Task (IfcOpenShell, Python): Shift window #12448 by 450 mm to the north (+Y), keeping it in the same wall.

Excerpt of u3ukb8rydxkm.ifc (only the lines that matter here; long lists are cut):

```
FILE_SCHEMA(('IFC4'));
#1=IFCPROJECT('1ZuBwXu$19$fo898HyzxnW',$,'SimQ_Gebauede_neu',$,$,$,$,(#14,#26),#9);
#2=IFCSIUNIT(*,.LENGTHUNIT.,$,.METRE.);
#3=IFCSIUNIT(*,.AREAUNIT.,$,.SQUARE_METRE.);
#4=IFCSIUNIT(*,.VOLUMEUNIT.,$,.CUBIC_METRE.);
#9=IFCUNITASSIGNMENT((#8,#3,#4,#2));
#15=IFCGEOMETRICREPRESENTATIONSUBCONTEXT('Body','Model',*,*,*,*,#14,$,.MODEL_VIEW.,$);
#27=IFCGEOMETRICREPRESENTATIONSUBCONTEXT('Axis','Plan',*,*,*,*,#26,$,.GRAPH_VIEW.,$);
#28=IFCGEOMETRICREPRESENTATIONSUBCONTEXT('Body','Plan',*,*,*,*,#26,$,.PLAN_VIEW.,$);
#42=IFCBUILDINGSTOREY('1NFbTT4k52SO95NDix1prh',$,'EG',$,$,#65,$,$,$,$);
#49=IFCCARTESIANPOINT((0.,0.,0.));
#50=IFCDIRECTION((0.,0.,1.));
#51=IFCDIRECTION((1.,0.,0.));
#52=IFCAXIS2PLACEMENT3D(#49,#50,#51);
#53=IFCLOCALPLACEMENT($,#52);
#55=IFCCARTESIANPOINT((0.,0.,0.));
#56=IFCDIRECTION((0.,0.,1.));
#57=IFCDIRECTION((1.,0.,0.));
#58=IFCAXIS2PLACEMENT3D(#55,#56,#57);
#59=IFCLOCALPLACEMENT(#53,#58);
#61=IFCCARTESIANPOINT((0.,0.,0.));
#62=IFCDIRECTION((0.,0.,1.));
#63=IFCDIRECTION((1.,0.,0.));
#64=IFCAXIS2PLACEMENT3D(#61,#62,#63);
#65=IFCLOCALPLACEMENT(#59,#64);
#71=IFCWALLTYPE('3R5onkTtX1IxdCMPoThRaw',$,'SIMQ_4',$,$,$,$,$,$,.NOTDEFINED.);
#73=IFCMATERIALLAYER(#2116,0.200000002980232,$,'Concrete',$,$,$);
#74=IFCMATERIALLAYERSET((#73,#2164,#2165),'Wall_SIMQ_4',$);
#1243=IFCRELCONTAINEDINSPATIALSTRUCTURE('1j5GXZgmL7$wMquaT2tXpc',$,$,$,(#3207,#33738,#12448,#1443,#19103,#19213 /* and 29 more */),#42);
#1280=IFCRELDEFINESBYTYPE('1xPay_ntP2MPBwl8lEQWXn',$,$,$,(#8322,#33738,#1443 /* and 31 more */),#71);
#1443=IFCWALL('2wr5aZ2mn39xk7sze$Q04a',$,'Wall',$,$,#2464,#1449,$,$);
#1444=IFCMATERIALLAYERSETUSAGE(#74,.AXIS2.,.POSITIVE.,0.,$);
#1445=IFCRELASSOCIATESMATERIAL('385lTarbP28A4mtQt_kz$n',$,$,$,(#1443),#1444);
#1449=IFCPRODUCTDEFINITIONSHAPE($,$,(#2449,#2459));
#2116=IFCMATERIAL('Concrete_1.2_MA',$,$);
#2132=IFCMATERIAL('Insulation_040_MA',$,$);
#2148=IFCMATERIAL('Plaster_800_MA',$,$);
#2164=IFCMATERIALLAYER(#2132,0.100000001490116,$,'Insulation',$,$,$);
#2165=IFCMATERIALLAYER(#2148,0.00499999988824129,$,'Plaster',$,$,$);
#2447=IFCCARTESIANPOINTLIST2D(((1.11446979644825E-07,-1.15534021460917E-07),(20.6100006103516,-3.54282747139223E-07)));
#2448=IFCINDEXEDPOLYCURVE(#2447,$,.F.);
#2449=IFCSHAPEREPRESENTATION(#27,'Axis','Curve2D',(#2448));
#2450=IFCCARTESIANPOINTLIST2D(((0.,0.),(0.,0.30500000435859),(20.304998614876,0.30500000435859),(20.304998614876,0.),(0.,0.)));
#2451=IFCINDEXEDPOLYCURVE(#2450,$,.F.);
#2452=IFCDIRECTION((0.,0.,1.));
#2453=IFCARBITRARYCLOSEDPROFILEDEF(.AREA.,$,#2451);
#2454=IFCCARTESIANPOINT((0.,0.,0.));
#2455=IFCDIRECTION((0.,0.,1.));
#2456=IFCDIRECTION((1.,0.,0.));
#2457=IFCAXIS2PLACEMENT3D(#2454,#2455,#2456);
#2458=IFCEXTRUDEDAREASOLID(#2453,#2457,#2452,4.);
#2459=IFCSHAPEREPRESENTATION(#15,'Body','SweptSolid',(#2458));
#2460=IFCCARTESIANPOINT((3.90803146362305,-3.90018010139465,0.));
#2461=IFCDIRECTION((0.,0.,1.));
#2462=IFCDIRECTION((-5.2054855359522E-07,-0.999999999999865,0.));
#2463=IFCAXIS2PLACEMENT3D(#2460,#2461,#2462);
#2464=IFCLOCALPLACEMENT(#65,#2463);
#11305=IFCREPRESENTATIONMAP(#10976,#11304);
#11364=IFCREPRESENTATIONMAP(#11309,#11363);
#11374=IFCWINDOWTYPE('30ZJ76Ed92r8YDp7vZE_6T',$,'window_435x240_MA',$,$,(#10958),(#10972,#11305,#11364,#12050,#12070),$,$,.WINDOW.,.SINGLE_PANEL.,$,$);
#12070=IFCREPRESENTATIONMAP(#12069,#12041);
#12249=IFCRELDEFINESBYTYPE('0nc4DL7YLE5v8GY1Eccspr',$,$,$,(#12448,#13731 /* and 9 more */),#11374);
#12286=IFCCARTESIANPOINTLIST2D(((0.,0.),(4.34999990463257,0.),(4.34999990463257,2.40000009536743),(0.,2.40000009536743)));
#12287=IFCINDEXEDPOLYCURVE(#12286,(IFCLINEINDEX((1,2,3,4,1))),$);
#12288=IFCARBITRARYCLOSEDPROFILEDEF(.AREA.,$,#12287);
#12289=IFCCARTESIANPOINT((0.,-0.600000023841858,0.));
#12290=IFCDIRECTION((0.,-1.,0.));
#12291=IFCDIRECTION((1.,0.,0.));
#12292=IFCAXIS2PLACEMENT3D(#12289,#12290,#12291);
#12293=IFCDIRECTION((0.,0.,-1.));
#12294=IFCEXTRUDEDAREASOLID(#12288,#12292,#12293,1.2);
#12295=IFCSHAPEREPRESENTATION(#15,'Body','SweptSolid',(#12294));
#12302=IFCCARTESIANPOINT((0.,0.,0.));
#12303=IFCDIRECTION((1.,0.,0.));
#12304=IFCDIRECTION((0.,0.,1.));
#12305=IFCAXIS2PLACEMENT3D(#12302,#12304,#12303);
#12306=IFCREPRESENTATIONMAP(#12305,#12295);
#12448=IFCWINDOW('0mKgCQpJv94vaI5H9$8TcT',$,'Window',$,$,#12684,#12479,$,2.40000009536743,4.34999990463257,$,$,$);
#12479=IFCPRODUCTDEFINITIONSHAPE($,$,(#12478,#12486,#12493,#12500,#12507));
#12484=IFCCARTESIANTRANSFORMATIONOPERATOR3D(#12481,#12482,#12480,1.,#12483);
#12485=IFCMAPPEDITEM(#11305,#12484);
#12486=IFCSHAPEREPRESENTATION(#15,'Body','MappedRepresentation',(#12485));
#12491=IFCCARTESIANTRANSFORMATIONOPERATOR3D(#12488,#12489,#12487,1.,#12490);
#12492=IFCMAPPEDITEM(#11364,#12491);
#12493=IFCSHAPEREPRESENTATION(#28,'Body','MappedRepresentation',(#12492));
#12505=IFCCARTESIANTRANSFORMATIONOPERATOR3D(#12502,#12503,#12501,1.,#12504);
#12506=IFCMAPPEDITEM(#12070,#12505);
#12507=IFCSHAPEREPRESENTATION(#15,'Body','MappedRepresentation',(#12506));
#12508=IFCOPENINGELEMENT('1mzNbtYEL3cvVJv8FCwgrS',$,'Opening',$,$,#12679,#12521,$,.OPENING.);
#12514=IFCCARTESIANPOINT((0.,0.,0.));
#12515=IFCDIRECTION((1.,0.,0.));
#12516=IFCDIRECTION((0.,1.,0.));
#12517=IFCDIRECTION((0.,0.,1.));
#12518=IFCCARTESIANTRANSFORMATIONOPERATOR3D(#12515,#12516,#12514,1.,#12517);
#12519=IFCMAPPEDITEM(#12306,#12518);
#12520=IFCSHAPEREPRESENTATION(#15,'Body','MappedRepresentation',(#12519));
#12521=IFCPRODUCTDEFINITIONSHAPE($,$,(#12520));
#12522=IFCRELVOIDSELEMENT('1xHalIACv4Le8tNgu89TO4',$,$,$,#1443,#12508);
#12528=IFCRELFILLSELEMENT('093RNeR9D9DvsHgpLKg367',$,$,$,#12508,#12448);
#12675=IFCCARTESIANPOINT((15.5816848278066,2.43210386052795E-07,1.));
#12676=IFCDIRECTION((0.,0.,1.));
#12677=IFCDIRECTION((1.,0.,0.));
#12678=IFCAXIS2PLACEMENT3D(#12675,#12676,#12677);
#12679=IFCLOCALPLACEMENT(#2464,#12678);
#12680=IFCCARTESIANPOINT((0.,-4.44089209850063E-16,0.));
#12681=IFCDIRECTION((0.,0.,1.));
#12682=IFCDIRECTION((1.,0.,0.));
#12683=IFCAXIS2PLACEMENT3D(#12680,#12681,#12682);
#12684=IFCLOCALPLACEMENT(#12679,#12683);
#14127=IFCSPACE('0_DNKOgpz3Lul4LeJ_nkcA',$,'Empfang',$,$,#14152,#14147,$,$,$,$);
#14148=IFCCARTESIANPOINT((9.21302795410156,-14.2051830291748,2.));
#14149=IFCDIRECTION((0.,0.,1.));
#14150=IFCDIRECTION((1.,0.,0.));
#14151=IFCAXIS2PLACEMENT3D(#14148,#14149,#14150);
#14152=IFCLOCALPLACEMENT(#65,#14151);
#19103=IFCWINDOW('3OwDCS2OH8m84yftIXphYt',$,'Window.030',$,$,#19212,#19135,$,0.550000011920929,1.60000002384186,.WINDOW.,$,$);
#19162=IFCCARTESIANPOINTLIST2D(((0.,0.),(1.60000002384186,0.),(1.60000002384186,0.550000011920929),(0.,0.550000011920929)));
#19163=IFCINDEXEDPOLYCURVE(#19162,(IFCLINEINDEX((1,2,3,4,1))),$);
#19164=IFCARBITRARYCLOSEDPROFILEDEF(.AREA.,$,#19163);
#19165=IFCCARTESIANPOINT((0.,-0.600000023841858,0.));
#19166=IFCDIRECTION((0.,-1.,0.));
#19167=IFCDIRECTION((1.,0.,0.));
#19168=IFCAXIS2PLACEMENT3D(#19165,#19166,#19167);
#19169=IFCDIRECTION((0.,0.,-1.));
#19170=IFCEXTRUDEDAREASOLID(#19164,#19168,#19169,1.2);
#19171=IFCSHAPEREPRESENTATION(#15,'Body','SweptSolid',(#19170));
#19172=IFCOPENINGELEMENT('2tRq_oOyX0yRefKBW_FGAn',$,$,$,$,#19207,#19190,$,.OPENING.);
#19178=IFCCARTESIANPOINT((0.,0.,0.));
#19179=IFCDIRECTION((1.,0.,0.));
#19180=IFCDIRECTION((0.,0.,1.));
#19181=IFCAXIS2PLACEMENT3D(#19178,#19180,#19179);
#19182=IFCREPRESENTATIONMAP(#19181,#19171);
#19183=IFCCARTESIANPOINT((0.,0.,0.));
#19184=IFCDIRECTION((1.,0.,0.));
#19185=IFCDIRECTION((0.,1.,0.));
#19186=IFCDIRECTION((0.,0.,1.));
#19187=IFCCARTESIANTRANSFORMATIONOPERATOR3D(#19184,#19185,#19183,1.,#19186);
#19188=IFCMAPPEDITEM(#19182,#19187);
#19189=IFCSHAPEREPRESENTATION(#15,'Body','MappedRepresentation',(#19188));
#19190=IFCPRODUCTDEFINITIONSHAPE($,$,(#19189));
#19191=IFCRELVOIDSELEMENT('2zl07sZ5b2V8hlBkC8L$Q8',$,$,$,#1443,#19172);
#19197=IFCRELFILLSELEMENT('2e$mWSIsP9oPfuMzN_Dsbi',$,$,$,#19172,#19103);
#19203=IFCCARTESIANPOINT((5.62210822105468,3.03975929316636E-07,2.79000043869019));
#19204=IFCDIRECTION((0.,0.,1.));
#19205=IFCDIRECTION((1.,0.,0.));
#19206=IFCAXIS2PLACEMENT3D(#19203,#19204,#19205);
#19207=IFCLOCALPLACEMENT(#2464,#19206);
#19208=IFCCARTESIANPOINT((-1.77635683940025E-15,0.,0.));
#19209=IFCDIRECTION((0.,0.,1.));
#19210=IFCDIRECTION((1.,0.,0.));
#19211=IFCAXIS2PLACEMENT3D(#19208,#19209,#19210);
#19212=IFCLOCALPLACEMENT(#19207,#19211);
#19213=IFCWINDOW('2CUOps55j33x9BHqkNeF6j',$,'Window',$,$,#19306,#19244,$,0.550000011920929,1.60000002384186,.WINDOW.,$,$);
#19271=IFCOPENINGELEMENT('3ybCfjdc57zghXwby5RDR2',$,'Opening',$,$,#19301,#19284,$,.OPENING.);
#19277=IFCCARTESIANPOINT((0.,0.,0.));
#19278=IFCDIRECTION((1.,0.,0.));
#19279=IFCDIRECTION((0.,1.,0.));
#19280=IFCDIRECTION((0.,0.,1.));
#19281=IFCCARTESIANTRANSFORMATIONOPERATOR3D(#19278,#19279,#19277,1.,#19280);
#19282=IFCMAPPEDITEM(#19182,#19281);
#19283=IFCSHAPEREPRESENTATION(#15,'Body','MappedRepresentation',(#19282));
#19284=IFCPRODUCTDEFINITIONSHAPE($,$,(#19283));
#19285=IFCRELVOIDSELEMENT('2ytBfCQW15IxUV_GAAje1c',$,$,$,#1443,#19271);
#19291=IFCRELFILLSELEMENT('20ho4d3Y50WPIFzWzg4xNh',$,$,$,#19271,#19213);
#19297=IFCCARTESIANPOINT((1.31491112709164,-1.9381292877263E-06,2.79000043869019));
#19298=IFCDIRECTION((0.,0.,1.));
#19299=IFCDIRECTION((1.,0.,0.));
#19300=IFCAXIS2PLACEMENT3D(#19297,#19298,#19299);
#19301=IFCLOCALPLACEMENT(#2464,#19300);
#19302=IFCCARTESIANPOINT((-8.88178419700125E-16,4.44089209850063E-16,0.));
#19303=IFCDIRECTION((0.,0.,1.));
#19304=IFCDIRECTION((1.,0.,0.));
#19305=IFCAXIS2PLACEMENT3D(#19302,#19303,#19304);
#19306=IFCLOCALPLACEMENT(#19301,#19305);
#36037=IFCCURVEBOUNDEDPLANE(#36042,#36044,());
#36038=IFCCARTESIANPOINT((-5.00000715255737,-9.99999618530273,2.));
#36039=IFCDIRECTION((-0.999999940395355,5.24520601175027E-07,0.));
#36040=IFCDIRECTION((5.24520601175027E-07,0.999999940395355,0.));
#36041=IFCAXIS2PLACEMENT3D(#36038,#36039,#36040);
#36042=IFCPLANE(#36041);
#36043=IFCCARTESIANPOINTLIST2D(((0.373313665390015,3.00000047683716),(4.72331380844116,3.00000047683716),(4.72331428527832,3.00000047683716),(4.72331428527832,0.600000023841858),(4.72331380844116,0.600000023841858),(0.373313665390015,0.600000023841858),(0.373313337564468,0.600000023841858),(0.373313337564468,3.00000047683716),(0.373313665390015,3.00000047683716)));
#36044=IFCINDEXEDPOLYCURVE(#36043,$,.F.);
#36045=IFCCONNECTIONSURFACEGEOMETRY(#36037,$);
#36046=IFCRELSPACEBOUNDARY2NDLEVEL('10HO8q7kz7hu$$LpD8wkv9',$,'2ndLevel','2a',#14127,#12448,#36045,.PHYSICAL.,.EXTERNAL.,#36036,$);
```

```python
import numpy as np
import ifcopenshell
import ifcopenshell.api.geometry
import ifcopenshell.util.placement
import ifcopenshell.util.unit

model = ifcopenshell.open("u3ukb8rydxkm.ifc")
unit_scale = ifcopenshell.util.unit.calculate_unit_scale(model)

window = model.by_id(12448)
opening = window.FillsVoids[0].RelatingOpeningElement
wall = opening.VoidsElements[0].RelatingBuildingElement

wall_matrix = ifcopenshell.util.placement.get_local_placement(wall.ObjectPlacement)
shift = wall_matrix[:3, 0] * -0.45 / unit_scale
before = ifcopenshell.util.placement.get_local_placement(window.ObjectPlacement)[:3, 3].copy()

# The window is placed relative to its opening, so it follows when the opening moves.
matrix = ifcopenshell.util.placement.get_local_placement(opening.ObjectPlacement)
matrix[:3, 3] += shift
ifcopenshell.api.geometry.edit_object_placement(
    model, product=opening, matrix=matrix, is_si=False, should_transform_children=True
)

# Space boundary surfaces are stored in each space's coordinates; move them too.
for rel in window.ProvidesBoundaries:
    if not rel.ConnectionGeometry:
        continue
    surface = rel.ConnectionGeometry.SurfaceOnRelatingElement.BasisSurface
    space_matrix = ifcopenshell.util.placement.get_local_placement(rel.RelatingSpace.ObjectPlacement)
    point = np.array(surface.Position.Location.Coordinates) + space_matrix[:3, :3].T @ shift
    surface.Position = model.createIfcAxis2Placement3D(
        model.createIfcCartesianPoint(point.tolist()), surface.Position.Axis, surface.Position.RefDirection
    )

after = ifcopenshell.util.placement.get_local_placement(window.ObjectPlacement)[:3, 3]
print("window moved by", (after - before).round(3) + 0.0)

model.write("u3ukb8rydxkm_v2.ifc")
```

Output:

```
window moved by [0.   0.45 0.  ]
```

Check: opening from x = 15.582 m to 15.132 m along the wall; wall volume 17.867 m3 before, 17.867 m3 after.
